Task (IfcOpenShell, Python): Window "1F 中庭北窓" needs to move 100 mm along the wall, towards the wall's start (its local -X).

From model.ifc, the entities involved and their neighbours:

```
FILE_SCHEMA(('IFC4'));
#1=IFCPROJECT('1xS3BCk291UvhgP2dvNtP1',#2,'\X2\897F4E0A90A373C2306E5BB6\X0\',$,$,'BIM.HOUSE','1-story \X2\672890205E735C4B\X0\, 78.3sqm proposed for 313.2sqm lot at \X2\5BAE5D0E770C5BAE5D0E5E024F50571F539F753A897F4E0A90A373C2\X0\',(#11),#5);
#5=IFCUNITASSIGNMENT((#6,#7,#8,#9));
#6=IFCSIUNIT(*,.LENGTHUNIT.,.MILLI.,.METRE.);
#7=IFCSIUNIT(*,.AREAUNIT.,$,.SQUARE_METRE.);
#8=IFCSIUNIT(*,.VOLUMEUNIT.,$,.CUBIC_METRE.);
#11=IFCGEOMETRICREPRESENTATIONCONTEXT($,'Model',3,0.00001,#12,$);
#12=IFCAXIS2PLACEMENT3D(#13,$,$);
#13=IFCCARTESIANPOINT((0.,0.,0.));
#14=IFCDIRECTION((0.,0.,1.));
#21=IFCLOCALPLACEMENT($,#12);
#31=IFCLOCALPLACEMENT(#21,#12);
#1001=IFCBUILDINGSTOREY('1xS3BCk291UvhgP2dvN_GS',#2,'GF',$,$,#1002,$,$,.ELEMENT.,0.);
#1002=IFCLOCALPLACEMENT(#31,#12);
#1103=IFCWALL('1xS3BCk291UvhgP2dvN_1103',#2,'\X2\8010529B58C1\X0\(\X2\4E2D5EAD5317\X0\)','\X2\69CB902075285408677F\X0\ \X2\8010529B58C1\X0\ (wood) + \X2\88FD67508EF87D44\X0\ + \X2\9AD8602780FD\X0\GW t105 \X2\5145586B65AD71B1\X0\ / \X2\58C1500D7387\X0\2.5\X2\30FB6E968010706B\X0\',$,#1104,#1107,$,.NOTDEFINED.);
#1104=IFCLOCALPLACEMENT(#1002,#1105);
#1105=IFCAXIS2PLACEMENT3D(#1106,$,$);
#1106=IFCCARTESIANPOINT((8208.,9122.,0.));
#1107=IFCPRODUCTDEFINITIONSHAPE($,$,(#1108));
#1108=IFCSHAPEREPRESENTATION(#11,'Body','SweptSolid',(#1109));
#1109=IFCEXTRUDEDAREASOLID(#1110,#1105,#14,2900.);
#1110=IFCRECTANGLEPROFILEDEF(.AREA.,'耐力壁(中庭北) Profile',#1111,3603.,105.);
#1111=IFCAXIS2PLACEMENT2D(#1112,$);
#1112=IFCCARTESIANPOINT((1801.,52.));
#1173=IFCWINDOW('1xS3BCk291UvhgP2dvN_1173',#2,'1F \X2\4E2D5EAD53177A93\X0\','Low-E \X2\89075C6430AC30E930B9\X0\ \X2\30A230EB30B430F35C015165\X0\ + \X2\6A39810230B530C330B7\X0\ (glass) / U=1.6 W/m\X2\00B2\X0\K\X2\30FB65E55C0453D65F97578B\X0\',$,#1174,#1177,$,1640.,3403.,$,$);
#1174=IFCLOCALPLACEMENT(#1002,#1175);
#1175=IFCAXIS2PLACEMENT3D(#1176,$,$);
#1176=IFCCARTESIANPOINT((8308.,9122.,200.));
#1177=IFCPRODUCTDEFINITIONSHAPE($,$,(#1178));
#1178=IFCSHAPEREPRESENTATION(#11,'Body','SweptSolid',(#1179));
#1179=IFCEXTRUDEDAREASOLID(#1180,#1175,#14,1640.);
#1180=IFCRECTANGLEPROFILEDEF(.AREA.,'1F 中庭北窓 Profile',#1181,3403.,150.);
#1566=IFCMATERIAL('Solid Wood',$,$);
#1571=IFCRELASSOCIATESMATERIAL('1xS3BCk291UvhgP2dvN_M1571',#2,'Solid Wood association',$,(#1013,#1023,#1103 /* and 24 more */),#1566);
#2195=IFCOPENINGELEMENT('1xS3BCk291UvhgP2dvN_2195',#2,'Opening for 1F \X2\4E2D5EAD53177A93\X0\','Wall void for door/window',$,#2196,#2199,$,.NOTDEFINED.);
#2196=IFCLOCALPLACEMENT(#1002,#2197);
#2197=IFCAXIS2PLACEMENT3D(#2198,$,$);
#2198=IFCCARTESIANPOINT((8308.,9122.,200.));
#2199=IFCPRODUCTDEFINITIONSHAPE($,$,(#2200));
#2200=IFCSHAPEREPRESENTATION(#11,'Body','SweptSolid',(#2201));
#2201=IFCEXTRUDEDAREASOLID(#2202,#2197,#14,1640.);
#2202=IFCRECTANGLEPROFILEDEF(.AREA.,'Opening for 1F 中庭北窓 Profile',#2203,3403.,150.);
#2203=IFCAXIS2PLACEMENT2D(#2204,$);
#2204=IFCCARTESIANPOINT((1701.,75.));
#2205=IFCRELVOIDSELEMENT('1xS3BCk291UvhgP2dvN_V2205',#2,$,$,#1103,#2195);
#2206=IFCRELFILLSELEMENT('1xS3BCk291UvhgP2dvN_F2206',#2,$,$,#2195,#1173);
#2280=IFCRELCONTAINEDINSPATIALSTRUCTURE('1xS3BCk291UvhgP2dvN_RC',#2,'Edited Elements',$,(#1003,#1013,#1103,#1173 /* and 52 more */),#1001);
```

```python
import ifcopenshell
import ifcopenshell.api.geometry
import ifcopenshell.util.placement

model = ifcopenshell.open("model.ifc")

window = model.by_guid("1xS3BCk291UvhgP2dvN_1173")
opening = window.FillsVoids[0].RelatingOpeningElement
wall = opening.VoidsElements[0].RelatingBuildingElement

wall_matrix = ifcopenshell.util.placement.get_local_placement(wall.ObjectPlacement)
shift = wall_matrix[:3, 0] * -100.0
before = ifcopenshell.util.placement.get_local_placement(window.ObjectPlacement)[:3, 3].copy()

# The window is not placed relative to its opening, so move both.
for product in (opening, window):
    matrix = ifcopenshell.util.placement.get_local_placement(product.ObjectPlacement)
    matrix[:3, 3] += shift
    ifcopenshell.api.geometry.edit_object_placement(model, product=product, matrix=matrix, is_si=False)

after = ifcopenshell.util.placement.get_local_placement(window.ObjectPlacement)[:3, 3]
print("window moved by", (after - before).round(3) + 0.0)

model.write("model_edited.ifc")
```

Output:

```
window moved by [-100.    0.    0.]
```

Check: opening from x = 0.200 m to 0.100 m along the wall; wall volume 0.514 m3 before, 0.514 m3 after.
